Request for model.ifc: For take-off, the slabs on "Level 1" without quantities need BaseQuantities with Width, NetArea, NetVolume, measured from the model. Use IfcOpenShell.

First a look at what the model holds.

```python
import ifcopenshell
import ifcopenshell.util.element
import ifcopenshell.util.unit

model = ifcopenshell.open("model.ifc")
print(model.schema)
for unit_type in ("LENGTHUNIT", "AREAUNIT", "VOLUMEUNIT"):
    print(unit_type, ifcopenshell.util.unit.calculate_unit_scale(model, unit_type))
storey = next(s for s in model.by_type("IfcBuildingStorey") if s.Name == "Level 1")
slabs = [e for e in ifcopenshell.util.element.get_decomposition(storey) if e.is_a("IfcSlab")]
for e in sorted(slabs, key=lambda e: e.id()):
    print(e.id(), e.is_a(), e.Name, list(ifcopenshell.util.element.get_psets(e, qtos_only=True)), sep=" | ")
```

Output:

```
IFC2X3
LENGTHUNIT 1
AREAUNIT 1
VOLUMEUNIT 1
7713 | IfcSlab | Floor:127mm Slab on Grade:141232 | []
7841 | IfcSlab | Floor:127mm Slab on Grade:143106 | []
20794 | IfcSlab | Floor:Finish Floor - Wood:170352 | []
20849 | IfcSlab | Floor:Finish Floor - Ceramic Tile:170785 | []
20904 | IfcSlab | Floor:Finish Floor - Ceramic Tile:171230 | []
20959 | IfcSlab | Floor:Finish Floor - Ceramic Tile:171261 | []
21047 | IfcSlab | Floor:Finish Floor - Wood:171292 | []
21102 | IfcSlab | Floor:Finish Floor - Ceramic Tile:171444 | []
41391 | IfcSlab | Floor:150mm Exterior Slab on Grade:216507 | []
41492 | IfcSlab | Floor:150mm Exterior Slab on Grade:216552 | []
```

```python
import ifcopenshell
import ifcopenshell.api.pset
import ifcopenshell.geom
import ifcopenshell.util.element
import ifcopenshell.util.shape
import ifcopenshell.util.unit

model = ifcopenshell.open("model.ifc")
unit_scale = ifcopenshell.util.unit.calculate_unit_scale(model)
area_scale = ifcopenshell.util.unit.calculate_unit_scale(model, "AREAUNIT")
volume_scale = ifcopenshell.util.unit.calculate_unit_scale(model, "VOLUMEUNIT")
settings = ifcopenshell.geom.settings()

storey = next(s for s in model.by_type("IfcBuildingStorey") if s.Name == "Level 1")
slabs = [e for e in ifcopenshell.util.element.get_decomposition(storey) if e.is_a("IfcSlab")]

for e in sorted(slabs, key=lambda e: e.id()):
    if ifcopenshell.util.element.get_psets(e, qtos_only=True, should_inherit=False):
        continue
    # Geometry comes back in metres, in the element's own axes.
    shape = ifcopenshell.geom.create_shape(settings, e)
    values = {
        "Width": ifcopenshell.util.shape.get_z(shape.geometry) / unit_scale,
        "NetArea": ifcopenshell.util.shape.get_footprint_area(shape.geometry) / area_scale,
        "NetVolume": ifcopenshell.util.shape.get_volume(shape.geometry) / volume_scale,
    }
    qto = ifcopenshell.api.pset.add_qto(model, product=e, name="BaseQuantities")
    ifcopenshell.api.pset.edit_qto(model, qto=qto, properties=values)
    print(e.id(), {k: round(v, 3) for k, v in values.items()})

model.write("model_v2.ifc")
```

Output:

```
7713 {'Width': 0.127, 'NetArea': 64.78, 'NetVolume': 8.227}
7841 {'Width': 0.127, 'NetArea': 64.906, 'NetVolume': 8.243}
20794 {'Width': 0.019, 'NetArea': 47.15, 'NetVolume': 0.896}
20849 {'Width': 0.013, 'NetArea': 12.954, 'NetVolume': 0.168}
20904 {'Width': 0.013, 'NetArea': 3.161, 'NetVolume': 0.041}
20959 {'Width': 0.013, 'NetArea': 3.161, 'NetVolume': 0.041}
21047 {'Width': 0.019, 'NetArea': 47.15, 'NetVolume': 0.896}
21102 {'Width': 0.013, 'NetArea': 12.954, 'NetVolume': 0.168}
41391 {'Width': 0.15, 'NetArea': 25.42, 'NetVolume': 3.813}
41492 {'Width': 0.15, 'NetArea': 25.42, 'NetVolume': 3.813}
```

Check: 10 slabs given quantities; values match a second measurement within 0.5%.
